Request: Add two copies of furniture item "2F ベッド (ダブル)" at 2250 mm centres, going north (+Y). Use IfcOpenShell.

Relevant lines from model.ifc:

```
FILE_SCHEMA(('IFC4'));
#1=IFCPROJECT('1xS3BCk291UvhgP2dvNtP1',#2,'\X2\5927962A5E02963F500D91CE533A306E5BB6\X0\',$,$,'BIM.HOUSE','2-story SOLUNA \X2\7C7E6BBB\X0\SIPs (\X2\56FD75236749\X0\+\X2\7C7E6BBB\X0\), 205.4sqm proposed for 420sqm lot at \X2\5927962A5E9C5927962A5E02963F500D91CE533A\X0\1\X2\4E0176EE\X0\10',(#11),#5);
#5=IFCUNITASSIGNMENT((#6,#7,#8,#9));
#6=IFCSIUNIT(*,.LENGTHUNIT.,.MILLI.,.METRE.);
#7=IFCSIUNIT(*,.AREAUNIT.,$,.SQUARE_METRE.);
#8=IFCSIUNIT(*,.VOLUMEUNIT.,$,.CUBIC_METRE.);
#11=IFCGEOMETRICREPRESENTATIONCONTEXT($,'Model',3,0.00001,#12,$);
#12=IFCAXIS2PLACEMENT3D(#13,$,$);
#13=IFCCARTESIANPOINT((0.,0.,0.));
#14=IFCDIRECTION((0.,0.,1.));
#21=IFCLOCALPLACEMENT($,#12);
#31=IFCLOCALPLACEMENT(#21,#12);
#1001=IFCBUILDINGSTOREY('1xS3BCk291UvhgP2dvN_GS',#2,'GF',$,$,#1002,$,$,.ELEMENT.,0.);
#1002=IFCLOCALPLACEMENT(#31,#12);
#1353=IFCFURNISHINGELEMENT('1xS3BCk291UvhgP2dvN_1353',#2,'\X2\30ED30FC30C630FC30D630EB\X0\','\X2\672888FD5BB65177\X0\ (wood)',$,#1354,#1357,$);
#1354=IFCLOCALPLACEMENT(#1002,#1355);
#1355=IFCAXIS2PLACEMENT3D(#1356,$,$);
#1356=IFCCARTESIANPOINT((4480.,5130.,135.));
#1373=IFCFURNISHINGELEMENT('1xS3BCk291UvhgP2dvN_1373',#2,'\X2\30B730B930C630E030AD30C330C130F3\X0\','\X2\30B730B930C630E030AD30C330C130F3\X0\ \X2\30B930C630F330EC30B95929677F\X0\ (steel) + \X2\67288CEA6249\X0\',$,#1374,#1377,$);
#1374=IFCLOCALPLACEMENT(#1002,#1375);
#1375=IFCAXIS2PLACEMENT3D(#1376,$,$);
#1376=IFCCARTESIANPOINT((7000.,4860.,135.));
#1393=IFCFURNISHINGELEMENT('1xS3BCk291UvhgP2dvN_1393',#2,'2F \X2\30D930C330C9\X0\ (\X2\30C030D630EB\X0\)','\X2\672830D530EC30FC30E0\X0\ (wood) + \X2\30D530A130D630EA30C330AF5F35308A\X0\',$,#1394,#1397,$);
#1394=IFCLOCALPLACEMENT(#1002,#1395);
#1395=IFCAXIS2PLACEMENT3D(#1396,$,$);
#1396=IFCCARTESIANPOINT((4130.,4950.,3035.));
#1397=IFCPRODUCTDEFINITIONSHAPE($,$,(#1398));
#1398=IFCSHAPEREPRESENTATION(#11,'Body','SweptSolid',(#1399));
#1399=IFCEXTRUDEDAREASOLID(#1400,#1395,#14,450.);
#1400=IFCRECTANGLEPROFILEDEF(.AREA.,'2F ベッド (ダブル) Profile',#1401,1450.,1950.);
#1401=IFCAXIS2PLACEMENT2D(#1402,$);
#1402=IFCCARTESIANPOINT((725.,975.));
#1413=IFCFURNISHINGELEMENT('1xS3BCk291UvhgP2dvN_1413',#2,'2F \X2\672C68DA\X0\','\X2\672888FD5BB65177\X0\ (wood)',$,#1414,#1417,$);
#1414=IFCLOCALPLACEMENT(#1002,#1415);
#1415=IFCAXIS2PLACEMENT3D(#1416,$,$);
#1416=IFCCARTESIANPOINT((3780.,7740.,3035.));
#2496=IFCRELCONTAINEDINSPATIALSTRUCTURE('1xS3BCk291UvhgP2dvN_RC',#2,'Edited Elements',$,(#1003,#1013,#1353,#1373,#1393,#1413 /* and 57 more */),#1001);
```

```python
import numpy as np
import ifcopenshell
import ifcopenshell.api.geometry
import ifcopenshell.api.root
import ifcopenshell.util.element
import ifcopenshell.util.placement
import ifcopenshell.util.unit

model = ifcopenshell.open("model.ifc")
unit_scale = ifcopenshell.util.unit.calculate_unit_scale(model)


def reuse_history(source, copy):
    """copy_class also copies each property set's owner history, people and application; keep the originals."""
    for rel in copy.IsDefinedBy:
        if rel.is_a("IfcRelDefinesByProperties") and (history := rel.RelatingPropertyDefinition.OwnerHistory):
            rel.RelatingPropertyDefinition.OwnerHistory = source.OwnerHistory
            ifcopenshell.util.element.remove_deep2(model, history)


source = model.by_guid("1xS3BCk291UvhgP2dvN_1393")
base = ifcopenshell.util.placement.get_local_placement(source.ObjectPlacement)
step = np.array([0.0, 1.0, 0.0]) * 2.25 / unit_scale

for i in range(1, 3):
    copy = ifcopenshell.api.root.copy_class(model, product=source)
    copy.Representation = ifcopenshell.util.element.copy_deep(
        model, source.Representation, exclude=["IfcGeometricRepresentationContext", "IfcRepresentationMap"]
    )
    reuse_history(source, copy)
    matrix = base.copy()
    matrix[:3, 3] += i * step
    print("added at", matrix[:3, 3].round(3) + 0.0)
    ifcopenshell.api.geometry.edit_object_placement(model, product=copy, matrix=matrix, is_si=False)

model.write("model-out.ifc")
```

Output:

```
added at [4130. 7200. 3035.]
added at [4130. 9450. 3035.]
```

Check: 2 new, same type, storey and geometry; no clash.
